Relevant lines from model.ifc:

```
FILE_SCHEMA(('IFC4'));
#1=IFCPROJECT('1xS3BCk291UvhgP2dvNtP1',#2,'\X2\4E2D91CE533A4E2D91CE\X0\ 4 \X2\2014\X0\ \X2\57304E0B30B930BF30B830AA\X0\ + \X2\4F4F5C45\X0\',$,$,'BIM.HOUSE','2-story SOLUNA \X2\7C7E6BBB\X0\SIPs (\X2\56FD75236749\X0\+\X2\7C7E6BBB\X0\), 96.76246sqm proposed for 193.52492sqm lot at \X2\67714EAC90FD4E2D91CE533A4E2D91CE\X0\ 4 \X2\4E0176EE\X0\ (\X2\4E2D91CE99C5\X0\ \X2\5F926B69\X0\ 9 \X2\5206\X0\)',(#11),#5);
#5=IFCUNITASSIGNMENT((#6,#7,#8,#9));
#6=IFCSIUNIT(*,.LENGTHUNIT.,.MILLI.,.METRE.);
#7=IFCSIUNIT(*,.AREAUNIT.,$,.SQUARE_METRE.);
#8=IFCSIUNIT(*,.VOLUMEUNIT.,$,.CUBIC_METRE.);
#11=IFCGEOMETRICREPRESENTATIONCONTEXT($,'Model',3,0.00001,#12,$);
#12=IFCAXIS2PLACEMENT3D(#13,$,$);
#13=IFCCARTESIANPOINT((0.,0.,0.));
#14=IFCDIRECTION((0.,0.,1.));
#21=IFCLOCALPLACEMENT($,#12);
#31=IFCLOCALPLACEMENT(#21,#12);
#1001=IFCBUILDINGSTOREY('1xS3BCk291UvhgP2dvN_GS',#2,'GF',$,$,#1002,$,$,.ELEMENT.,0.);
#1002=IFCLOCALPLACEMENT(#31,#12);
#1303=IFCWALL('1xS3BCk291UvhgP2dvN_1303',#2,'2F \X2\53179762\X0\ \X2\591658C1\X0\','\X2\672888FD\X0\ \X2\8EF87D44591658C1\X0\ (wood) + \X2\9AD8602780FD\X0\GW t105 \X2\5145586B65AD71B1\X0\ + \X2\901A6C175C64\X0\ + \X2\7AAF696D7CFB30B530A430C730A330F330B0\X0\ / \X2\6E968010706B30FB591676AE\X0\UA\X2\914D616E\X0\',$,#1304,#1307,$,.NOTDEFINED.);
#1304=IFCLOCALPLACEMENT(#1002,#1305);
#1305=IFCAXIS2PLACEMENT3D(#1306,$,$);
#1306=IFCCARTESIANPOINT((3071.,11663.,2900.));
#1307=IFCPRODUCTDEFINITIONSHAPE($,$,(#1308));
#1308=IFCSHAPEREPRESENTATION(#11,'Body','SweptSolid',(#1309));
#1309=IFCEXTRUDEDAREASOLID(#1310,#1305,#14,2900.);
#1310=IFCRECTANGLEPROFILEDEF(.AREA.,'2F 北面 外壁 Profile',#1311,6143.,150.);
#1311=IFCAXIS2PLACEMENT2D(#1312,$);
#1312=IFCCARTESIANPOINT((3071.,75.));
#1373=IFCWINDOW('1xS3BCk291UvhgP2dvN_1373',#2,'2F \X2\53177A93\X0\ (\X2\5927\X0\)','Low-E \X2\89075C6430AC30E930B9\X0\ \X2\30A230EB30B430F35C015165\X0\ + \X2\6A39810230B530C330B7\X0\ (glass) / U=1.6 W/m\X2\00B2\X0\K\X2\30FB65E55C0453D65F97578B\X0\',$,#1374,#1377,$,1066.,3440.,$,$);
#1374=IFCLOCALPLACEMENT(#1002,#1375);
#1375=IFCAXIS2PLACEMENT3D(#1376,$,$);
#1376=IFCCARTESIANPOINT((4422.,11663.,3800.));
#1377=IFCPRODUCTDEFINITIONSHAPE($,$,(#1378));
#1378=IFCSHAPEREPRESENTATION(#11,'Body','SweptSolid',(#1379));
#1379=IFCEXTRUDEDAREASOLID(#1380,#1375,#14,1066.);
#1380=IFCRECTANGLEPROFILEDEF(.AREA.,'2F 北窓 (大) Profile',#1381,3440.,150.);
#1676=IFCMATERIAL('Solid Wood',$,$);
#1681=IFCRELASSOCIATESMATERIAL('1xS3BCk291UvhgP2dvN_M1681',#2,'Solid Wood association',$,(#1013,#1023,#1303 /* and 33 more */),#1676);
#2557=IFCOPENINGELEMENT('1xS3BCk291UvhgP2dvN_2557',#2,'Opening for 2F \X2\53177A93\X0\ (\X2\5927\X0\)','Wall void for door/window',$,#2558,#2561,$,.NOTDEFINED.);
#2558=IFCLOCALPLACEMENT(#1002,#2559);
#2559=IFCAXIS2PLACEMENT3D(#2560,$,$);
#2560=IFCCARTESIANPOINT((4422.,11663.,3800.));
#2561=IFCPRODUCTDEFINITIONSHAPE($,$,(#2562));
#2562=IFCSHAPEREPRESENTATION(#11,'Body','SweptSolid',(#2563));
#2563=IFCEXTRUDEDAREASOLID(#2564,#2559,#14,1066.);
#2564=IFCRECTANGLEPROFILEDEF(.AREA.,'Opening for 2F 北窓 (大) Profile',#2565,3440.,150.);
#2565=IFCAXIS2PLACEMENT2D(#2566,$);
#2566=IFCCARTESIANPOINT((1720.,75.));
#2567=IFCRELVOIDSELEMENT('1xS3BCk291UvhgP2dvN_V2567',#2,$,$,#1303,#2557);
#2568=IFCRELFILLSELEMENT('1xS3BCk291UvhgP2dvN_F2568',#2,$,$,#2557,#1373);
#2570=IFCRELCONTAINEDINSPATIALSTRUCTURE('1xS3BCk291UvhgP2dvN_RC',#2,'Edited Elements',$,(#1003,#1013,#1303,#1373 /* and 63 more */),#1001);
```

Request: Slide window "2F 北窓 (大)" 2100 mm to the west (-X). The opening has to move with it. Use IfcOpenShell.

```python
import ifcopenshell
import ifcopenshell.api.geometry
import ifcopenshell.util.placement
import ifcopenshell.util.unit

model = ifcopenshell.open("model.ifc")
unit_scale = ifcopenshell.util.unit.calculate_unit_scale(model)

window = model.by_guid("1xS3BCk291UvhgP2dvN_1373")
opening = window.FillsVoids[0].RelatingOpeningElement
wall = opening.VoidsElements[0].RelatingBuildingElement

wall_matrix = ifcopenshell.util.placement.get_local_placement(wall.ObjectPlacement)
shift = wall_matrix[:3, 0] * -2.1 / unit_scale
before = ifcopenshell.util.placement.get_local_placement(window.ObjectPlacement)[:3, 3].copy()

# The window is not placed relative to its opening, so move both.
for product in (opening, window):
    matrix = ifcopenshell.util.placement.get_local_placement(product.ObjectPlacement)
    matrix[:3, 3] += shift
    ifcopenshell.api.geometry.edit_object_placement(model, product=product, matrix=matrix, is_si=False)

after = ifcopenshell.util.placement.get_local_placement(window.ObjectPlacement)[:3, 3]
print("window moved by", (after - before).round(3) + 0.0)

model.write("model_v2.ifc")
```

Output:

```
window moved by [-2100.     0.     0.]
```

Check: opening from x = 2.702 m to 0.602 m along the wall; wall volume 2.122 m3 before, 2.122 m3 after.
